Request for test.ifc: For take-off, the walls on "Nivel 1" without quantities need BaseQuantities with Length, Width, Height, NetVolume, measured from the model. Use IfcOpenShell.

First a look at what the model holds.

```python
import ifcopenshell
import ifcopenshell.util.element
import ifcopenshell.util.unit

model = ifcopenshell.open("test.ifc")
print(model.schema)
for unit_type in ("LENGTHUNIT", "AREAUNIT", "VOLUMEUNIT"):
    print(unit_type, ifcopenshell.util.unit.calculate_unit_scale(model, unit_type))
storey = next(s for s in model.by_type("IfcBuildingStorey") if s.Name == "Nivel 1")
walls = [e for e in ifcopenshell.util.element.get_decomposition(storey) if e.is_a("IfcWall")]
for e in sorted(walls, key=lambda e: e.id()):
    print(e.id(), e.is_a(), e.Name, list(ifcopenshell.util.element.get_psets(e, qtos_only=True)), sep=" | ")
```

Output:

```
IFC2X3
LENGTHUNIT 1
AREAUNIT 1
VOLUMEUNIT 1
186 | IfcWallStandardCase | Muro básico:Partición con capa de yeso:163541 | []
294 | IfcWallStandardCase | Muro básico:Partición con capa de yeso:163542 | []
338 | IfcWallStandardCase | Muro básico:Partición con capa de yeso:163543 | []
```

```python
import ifcopenshell
import ifcopenshell.api.pset
import ifcopenshell.geom
import ifcopenshell.util.element
import ifcopenshell.util.shape
import ifcopenshell.util.unit

model = ifcopenshell.open("test.ifc")
unit_scale = ifcopenshell.util.unit.calculate_unit_scale(model)
volume_scale = ifcopenshell.util.unit.calculate_unit_scale(model, "VOLUMEUNIT")
settings = ifcopenshell.geom.settings()

storey = next(s for s in model.by_type("IfcBuildingStorey") if s.Name == "Nivel 1")
walls = [e for e in ifcopenshell.util.element.get_decomposition(storey) if e.is_a("IfcWall")]

for e in sorted(walls, key=lambda e: e.id()):
    if ifcopenshell.util.element.get_psets(e, qtos_only=True, should_inherit=False):
        continue
    # Geometry comes back in metres, in the element's own axes.
    shape = ifcopenshell.geom.create_shape(settings, e)
    values = {
        "Length": ifcopenshell.util.shape.get_x(shape.geometry) / unit_scale,
        "Width": ifcopenshell.util.shape.get_y(shape.geometry) / unit_scale,
        "Height": ifcopenshell.util.shape.get_z(shape.geometry) / unit_scale,
        "NetVolume": ifcopenshell.util.shape.get_volume(shape.geometry) / volume_scale,
    }
    qto = ifcopenshell.api.pset.add_qto(model, product=e, name="BaseQuantities")
    ifcopenshell.api.pset.edit_qto(model, qto=qto, properties=values)
    print(e.id(), {k: round(v, 3) for k, v in values.items()})

model.write("test_v2.ifc")
```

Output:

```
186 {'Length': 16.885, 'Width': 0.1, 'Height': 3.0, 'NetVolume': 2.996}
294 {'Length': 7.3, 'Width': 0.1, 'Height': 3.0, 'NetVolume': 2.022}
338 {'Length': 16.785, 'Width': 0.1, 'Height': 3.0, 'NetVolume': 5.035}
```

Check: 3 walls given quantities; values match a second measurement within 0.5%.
